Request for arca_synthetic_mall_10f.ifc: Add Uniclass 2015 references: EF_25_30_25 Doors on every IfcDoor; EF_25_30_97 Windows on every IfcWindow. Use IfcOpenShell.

First a look at what the model holds.

```python
import ifcopenshell

model = ifcopenshell.open("arca_synthetic_mall_10f.ifc")
print(model.schema)
print("classifications:", [c.Name for c in model.by_type("IfcClassification")])
for ifc_class in ("IfcDoor", "IfcRoof", "IfcStair", "IfcWall", "IfcWindow"):
    print(ifc_class, len(model.by_type(ifc_class)))
```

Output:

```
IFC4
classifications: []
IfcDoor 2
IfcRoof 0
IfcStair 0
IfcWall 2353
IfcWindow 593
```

```python
import ifcopenshell
import ifcopenshell.api.classification

model = ifcopenshell.open("arca_synthetic_mall_10f.ifc")

system = ifcopenshell.api.classification.add_classification(model, classification="Uniclass 2015")

codes = {
    "IfcDoor": ("EF_25_30_25", "Doors"),
    "IfcWindow": ("EF_25_30_97", "Windows"),
}
for ifc_class, (code, name) in codes.items():
    products = model.by_type(ifc_class)
    ifcopenshell.api.classification.add_reference(
        model, products=products, classification=system, identification=code, name=name
    )
    print(code, len(products))

model.write("arca_synthetic_mall_10f_updated.ifc")
```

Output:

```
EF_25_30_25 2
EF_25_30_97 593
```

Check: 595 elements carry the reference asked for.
